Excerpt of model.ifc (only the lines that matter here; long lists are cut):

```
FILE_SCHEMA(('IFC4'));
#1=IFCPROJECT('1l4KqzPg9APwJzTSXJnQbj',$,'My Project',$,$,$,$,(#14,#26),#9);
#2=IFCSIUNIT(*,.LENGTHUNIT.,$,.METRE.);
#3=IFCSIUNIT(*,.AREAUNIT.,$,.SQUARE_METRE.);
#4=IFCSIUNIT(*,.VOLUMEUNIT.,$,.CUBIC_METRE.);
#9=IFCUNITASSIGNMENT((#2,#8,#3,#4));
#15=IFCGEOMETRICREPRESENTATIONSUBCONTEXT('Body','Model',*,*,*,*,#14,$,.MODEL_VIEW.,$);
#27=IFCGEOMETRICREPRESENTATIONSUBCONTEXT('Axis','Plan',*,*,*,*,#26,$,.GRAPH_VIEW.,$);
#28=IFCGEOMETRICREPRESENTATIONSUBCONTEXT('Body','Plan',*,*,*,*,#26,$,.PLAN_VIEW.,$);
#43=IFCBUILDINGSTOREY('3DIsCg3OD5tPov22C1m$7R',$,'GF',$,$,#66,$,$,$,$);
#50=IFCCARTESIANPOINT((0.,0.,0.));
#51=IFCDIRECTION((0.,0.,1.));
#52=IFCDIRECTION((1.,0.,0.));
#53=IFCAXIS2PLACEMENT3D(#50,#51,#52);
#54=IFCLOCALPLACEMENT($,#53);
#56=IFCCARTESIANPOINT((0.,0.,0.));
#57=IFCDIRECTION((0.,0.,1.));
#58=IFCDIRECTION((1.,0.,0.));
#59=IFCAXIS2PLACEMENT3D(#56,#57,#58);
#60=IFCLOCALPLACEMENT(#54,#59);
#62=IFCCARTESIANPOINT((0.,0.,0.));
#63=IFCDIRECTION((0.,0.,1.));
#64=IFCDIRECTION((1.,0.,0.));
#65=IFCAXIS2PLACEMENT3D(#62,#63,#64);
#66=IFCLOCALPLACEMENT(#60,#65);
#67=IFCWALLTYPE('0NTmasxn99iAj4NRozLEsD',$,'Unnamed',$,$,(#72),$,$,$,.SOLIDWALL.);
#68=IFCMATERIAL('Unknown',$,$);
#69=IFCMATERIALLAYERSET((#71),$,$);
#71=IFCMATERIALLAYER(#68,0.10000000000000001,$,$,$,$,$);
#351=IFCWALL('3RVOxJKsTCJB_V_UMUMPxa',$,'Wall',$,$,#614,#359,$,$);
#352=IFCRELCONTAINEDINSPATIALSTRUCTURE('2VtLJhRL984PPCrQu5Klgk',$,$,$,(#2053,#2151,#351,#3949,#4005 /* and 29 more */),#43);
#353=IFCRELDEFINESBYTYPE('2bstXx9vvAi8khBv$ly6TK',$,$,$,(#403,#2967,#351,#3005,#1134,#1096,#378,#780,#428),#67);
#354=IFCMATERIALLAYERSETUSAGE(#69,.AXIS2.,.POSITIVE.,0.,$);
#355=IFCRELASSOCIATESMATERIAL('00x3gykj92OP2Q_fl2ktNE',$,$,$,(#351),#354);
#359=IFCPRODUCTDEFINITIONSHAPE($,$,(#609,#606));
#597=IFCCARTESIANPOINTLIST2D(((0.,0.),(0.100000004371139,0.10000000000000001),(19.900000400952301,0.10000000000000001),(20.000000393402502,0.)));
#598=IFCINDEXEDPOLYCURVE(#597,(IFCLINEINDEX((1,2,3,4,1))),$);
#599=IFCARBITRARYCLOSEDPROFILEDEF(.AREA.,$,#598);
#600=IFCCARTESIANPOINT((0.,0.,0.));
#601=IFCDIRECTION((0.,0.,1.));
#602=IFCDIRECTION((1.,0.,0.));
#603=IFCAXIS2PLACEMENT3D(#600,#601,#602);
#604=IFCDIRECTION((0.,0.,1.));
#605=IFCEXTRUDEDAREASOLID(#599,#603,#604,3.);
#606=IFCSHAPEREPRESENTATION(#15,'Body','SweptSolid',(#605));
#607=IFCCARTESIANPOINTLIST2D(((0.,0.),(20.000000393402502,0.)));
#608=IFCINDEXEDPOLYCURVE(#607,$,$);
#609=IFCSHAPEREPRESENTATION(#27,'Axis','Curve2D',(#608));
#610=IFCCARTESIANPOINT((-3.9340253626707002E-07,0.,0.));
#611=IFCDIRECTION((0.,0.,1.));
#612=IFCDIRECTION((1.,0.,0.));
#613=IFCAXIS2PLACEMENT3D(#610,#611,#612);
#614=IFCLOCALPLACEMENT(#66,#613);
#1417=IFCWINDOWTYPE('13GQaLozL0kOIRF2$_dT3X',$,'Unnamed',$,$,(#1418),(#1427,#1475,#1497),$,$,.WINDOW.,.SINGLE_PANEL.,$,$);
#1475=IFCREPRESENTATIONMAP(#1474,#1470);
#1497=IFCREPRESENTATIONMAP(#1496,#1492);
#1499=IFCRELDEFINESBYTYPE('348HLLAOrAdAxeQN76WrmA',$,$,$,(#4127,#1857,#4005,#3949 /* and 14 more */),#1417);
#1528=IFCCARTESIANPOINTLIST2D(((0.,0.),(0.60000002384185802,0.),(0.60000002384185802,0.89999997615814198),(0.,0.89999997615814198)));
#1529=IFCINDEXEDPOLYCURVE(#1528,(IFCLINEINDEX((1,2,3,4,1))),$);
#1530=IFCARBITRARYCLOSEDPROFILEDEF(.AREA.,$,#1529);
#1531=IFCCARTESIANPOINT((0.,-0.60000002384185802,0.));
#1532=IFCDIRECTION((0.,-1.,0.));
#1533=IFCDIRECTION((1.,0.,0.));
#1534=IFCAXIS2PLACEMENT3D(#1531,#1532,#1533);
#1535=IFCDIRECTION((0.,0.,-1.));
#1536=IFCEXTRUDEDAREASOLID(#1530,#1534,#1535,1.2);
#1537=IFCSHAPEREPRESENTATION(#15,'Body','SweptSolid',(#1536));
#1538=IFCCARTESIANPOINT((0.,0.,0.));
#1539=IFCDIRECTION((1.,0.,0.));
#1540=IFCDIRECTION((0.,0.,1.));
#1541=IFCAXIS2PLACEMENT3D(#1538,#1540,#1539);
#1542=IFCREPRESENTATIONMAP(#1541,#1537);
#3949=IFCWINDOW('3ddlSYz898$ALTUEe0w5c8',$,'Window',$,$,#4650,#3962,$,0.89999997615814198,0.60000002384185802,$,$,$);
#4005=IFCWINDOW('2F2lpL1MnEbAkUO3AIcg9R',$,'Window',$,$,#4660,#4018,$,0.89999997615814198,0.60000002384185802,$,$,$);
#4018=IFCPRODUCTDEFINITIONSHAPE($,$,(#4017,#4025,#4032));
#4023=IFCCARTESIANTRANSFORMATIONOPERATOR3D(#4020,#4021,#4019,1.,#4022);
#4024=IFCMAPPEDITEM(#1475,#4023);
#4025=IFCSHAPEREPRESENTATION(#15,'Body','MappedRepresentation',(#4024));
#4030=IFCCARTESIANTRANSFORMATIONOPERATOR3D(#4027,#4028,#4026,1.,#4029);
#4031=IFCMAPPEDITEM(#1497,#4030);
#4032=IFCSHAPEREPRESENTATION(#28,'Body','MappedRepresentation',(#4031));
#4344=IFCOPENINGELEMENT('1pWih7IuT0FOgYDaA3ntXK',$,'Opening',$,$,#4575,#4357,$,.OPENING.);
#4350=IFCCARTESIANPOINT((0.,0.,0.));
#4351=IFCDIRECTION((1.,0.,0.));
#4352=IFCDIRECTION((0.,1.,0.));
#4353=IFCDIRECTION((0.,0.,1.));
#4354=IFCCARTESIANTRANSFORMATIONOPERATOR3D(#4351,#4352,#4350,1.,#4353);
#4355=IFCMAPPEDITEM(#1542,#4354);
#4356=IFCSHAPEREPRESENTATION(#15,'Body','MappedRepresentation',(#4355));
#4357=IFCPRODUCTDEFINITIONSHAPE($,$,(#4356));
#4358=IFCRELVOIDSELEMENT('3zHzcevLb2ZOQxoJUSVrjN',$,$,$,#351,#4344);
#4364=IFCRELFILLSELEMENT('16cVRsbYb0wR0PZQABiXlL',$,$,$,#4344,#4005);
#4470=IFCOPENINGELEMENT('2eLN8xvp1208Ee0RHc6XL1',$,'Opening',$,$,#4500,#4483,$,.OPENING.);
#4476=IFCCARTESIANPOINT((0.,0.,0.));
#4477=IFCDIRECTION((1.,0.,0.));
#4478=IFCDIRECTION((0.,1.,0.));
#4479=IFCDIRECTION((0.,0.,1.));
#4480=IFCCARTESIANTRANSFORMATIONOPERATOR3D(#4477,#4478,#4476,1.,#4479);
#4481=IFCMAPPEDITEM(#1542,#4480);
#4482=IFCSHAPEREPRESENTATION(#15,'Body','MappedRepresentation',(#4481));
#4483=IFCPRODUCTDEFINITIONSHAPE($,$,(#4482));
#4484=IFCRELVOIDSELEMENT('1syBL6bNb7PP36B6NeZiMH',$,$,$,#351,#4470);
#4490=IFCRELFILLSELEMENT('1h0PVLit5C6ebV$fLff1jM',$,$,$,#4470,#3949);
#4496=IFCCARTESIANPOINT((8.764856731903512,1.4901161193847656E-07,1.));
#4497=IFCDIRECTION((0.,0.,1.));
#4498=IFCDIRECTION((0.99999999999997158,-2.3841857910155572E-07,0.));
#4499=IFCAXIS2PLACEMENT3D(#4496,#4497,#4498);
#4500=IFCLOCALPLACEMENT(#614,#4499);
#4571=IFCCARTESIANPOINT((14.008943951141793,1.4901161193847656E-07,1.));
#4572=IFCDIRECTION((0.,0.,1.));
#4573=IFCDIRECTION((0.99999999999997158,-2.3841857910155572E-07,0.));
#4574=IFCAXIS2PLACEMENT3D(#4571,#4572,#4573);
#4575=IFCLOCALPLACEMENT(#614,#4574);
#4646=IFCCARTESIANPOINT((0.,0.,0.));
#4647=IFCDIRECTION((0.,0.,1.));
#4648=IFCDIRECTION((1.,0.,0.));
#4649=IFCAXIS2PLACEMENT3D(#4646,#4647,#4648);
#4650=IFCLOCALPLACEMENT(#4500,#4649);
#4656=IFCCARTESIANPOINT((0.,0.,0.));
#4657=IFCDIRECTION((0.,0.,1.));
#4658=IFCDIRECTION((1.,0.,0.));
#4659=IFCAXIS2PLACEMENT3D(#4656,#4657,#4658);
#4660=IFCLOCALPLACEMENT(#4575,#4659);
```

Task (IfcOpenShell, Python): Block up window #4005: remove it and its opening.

```python
import ifcopenshell
import ifcopenshell.api.feature
import ifcopenshell.api.root
import ifcopenshell.geom
import ifcopenshell.util.shape

model = ifcopenshell.open("model.ifc")
settings = ifcopenshell.geom.settings()


def volume(element):
    """Net volume in cubic metres, openings subtracted."""
    shape = ifcopenshell.geom.create_shape(settings, element)
    return ifcopenshell.util.shape.get_volume(shape.geometry)


window = model.by_guid("2F2lpL1MnEbAkUO3AIcg9R")
opening = window.FillsVoids[0].RelatingOpeningElement
wall = opening.VoidsElements[0].RelatingBuildingElement
before = volume(wall)

ifcopenshell.api.root.remove_product(model, product=window)
ifcopenshell.api.feature.remove_feature(model, feature=opening)

after = volume(wall)

print(f"wall volume {before:.3f} -> {after:.3f} m3")

model.write("model-out.ifc")
```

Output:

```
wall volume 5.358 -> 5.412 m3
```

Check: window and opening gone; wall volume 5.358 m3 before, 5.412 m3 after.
